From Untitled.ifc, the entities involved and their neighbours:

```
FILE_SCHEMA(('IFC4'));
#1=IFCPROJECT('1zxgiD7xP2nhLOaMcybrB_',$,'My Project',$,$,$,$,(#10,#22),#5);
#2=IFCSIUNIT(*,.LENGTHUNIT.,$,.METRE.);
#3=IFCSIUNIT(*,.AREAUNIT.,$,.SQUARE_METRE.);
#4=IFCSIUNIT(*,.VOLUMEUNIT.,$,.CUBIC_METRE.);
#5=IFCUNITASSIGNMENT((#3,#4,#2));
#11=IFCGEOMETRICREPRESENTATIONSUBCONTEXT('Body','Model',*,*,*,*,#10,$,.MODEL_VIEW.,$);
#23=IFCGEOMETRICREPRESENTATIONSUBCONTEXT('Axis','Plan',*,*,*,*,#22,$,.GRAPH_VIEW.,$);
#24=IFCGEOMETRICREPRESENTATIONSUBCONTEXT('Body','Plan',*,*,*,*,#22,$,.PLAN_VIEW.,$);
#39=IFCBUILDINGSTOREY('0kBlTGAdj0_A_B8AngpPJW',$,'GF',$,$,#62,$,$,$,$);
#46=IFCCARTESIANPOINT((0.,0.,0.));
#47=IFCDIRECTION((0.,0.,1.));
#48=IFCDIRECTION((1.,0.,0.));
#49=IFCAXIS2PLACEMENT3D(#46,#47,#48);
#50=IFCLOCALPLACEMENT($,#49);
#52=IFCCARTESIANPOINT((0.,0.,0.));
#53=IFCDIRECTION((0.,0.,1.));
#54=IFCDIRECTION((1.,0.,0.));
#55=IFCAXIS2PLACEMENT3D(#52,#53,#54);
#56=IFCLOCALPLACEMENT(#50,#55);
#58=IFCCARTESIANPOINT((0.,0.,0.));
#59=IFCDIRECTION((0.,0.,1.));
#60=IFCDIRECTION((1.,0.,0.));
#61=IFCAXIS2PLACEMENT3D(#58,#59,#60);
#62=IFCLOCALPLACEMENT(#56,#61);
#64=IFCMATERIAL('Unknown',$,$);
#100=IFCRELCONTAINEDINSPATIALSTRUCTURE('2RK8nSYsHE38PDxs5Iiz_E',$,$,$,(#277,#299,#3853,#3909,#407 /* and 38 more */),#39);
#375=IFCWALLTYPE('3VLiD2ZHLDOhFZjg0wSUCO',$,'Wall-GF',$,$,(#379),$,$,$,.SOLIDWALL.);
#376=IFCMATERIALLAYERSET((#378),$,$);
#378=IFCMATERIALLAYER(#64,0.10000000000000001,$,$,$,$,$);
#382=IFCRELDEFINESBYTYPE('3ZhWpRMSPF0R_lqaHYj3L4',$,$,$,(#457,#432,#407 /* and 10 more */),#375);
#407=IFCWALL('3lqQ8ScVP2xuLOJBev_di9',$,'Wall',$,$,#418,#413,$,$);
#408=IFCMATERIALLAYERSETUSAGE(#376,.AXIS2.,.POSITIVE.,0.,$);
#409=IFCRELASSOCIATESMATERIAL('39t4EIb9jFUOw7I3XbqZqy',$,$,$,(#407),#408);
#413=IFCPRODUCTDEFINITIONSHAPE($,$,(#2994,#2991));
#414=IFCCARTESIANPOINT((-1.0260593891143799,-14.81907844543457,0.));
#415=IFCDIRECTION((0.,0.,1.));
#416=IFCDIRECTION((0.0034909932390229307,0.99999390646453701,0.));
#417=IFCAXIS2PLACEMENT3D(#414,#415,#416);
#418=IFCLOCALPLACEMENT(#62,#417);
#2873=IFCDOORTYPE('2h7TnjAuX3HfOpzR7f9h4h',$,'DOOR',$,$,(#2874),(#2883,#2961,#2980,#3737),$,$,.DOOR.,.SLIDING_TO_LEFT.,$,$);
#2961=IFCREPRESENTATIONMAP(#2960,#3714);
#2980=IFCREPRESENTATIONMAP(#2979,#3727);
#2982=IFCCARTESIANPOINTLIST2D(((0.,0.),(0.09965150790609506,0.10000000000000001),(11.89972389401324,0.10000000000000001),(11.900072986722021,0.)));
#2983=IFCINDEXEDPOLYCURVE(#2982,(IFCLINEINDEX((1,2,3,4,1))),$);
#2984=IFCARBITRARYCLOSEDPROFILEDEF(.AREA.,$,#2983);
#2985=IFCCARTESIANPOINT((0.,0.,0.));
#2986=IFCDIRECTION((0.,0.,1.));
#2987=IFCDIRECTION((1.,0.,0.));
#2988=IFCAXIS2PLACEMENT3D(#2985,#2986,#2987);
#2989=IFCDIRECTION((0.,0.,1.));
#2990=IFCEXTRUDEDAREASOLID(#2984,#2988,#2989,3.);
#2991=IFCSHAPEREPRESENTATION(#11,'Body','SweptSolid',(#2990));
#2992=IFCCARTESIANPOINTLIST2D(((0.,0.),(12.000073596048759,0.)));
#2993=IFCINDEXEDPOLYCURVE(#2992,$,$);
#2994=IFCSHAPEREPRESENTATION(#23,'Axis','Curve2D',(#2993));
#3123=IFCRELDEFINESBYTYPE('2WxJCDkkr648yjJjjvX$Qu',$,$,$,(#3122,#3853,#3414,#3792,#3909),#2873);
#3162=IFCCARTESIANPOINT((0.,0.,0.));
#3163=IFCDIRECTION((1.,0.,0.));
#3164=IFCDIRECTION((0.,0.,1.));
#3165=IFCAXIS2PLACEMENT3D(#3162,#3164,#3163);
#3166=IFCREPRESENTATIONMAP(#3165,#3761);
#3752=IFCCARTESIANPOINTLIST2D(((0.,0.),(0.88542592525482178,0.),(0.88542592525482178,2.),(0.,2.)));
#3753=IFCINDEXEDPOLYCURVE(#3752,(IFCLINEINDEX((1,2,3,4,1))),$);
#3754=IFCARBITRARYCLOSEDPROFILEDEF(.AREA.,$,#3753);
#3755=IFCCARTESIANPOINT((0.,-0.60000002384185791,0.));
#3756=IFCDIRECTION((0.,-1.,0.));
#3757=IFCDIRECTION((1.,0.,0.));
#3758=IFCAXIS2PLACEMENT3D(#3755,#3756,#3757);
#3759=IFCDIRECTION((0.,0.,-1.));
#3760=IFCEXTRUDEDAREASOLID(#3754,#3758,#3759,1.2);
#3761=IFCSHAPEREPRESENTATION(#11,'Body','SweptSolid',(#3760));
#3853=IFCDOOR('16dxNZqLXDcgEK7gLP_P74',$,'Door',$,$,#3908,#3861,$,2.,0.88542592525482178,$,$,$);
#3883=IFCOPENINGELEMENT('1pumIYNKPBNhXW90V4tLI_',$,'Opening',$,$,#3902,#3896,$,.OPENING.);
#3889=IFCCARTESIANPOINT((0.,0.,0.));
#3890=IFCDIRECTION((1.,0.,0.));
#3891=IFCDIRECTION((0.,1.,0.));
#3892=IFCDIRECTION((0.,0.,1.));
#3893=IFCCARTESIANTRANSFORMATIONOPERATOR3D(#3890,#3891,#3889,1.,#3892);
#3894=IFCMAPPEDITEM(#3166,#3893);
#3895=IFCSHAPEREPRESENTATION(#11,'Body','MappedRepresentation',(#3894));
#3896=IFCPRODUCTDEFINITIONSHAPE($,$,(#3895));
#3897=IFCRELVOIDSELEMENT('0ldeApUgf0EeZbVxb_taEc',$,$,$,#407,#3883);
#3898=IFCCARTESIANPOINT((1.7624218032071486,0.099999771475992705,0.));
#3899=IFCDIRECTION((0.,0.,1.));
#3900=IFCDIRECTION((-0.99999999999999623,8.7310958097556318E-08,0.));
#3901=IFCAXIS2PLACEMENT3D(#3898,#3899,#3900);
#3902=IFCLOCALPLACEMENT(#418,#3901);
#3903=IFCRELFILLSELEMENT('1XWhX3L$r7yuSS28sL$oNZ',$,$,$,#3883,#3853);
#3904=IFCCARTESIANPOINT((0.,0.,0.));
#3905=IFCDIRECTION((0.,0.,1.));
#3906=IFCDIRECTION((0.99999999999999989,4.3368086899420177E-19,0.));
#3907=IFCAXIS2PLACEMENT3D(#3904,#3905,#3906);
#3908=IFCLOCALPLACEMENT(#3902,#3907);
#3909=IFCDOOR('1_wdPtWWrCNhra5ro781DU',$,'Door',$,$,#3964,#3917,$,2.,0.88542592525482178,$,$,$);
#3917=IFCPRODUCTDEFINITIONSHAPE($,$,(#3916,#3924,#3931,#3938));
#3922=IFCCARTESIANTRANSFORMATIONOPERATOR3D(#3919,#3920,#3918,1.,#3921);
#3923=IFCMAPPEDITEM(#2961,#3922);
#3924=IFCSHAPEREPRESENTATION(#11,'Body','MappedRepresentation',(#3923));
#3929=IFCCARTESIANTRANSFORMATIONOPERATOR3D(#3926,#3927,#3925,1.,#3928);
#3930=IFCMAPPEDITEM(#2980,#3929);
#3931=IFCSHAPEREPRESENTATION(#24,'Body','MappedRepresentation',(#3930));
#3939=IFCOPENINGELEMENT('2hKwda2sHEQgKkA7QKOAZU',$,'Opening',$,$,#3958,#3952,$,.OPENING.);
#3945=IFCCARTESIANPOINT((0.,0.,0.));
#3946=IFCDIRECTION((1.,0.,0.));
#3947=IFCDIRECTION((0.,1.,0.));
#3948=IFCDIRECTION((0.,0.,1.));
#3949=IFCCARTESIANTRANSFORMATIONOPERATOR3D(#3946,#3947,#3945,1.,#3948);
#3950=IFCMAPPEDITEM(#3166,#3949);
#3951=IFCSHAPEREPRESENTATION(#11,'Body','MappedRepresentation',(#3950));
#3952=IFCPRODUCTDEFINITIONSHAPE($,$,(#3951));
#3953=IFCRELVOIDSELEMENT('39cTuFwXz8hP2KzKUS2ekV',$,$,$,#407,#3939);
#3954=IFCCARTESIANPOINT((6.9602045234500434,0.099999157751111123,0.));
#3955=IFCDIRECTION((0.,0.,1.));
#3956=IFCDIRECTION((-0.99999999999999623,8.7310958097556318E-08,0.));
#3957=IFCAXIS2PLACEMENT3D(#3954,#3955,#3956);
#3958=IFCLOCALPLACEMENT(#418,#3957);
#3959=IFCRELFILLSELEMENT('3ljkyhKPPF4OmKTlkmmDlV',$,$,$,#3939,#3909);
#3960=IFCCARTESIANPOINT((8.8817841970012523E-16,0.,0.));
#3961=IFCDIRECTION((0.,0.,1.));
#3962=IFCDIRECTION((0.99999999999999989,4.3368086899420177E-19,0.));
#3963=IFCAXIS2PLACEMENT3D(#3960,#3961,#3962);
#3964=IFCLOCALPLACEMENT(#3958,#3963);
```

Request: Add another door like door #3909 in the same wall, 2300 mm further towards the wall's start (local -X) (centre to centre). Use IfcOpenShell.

```python
import ifcopenshell
import ifcopenshell.api.feature
import ifcopenshell.api.geometry
import ifcopenshell.api.root
import ifcopenshell.geom
import ifcopenshell.util.element
import ifcopenshell.util.placement
import ifcopenshell.util.shape

model = ifcopenshell.open("Untitled.ifc")
settings = ifcopenshell.geom.settings()


def volume(element):
    """Net volume in cubic metres, openings subtracted."""
    shape = ifcopenshell.geom.create_shape(settings, element)
    return ifcopenshell.util.shape.get_volume(shape.geometry)


door = model.by_guid("1_wdPtWWrCNhra5ro781DU")
opening = door.FillsVoids[0].RelatingOpeningElement
wall = opening.VoidsElements[0].RelatingBuildingElement
before = volume(wall)
shift = ifcopenshell.util.placement.get_local_placement(wall.ObjectPlacement)[:3, 0] * -2.3

# copy_class copies the void relationship, type, container and properties, but no geometry.
new_opening = ifcopenshell.api.root.copy_class(model, product=opening)
new_opening.Representation = ifcopenshell.util.element.copy_deep(
    model, opening.Representation, exclude=["IfcGeometricRepresentationContext", "IfcRepresentationMap"]
)
new_door = ifcopenshell.api.root.copy_class(model, product=door)
new_door.Representation = ifcopenshell.util.element.copy_deep(
    model, door.Representation, exclude=["IfcGeometricRepresentationContext", "IfcRepresentationMap"]
)
ifcopenshell.api.feature.add_filling(model, opening=new_opening, element=new_door)

for old, new in ((opening, new_opening), (door, new_door)):
    matrix = ifcopenshell.util.placement.get_local_placement(old.ObjectPlacement)
    matrix[:3, 3] += shift
    ifcopenshell.api.geometry.edit_object_placement(model, product=new, matrix=matrix, is_si=False)

after = volume(wall)

print(f"wall volume {before:.3f} -> {after:.3f} m3")

model.write("Untitled-out.ifc")
```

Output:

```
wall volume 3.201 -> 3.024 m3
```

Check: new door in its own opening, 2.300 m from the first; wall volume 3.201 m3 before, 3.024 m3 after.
